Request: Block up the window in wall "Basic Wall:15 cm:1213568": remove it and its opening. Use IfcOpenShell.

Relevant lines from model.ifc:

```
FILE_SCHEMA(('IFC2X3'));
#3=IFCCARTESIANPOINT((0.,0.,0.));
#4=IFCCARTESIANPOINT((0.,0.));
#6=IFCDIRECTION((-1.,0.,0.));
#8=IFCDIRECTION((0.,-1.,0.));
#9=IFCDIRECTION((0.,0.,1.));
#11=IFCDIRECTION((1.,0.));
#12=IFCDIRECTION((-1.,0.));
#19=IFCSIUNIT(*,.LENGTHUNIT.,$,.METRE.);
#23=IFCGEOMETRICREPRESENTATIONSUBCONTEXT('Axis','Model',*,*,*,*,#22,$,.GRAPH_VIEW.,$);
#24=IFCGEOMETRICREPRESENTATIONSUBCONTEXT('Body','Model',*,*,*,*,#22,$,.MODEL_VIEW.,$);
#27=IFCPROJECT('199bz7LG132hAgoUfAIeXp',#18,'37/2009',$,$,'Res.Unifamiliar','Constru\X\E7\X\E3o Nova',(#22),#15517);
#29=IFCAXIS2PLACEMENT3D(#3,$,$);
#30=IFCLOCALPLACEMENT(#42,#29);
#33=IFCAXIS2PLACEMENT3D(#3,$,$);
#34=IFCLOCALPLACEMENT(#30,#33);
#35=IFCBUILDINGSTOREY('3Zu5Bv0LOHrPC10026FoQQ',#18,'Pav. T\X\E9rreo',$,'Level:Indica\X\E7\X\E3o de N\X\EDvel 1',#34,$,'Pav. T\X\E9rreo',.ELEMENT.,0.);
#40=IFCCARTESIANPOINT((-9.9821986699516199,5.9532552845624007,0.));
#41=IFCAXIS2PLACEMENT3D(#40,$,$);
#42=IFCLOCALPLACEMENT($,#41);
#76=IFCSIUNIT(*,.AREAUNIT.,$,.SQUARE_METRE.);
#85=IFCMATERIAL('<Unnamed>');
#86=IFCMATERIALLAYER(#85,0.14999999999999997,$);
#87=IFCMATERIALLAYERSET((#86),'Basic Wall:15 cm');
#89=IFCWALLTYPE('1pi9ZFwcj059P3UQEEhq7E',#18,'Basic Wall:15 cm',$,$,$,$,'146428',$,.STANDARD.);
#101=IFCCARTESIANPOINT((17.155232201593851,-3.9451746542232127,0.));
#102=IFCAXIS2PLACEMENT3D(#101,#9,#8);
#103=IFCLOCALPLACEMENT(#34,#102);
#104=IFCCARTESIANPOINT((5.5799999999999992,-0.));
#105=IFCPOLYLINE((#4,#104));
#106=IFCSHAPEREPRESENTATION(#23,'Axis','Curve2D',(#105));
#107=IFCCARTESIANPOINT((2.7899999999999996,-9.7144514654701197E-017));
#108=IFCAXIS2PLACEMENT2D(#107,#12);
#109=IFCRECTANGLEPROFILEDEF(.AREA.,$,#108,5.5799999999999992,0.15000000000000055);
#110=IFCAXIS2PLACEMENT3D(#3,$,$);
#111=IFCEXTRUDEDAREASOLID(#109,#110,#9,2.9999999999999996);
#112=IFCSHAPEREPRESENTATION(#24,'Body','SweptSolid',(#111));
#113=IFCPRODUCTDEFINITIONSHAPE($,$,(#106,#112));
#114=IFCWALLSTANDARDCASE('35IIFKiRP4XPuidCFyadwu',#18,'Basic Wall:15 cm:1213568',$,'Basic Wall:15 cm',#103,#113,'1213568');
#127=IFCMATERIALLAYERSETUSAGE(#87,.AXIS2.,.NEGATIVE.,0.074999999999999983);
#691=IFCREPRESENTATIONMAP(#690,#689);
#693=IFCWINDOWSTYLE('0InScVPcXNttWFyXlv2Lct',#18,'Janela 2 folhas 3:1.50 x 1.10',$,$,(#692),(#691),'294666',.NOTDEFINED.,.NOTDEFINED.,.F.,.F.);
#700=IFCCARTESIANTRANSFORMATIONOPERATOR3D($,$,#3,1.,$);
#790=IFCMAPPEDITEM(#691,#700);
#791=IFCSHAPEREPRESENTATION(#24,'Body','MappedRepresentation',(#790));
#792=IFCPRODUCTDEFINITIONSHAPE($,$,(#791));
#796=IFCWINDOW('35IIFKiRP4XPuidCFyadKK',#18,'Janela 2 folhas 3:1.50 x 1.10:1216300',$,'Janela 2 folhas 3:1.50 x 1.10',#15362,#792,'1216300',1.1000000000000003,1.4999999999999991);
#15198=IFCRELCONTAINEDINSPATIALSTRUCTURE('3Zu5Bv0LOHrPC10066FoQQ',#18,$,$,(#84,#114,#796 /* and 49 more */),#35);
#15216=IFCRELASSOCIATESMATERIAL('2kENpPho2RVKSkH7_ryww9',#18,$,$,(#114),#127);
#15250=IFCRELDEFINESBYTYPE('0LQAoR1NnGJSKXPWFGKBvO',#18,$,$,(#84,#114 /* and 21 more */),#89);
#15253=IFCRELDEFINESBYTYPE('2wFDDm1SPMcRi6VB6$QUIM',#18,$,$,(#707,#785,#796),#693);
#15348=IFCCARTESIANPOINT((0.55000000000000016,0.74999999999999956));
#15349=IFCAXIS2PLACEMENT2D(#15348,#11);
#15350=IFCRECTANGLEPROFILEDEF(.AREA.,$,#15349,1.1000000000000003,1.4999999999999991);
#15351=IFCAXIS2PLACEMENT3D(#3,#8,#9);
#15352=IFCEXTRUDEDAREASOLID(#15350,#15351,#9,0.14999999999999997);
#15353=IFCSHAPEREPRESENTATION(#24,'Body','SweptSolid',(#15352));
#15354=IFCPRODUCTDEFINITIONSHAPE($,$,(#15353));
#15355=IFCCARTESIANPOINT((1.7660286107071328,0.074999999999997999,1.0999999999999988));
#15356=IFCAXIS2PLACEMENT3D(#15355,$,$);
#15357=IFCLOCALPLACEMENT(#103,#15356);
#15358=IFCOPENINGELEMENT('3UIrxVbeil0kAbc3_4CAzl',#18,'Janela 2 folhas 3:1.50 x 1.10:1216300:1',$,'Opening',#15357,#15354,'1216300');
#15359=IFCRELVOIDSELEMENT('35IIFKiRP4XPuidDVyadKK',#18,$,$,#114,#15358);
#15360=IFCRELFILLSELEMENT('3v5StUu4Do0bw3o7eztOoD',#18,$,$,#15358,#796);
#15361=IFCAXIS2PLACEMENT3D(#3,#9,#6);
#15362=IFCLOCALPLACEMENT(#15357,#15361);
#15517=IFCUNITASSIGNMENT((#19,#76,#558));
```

```python
import ifcopenshell
import ifcopenshell.api.feature
import ifcopenshell.api.root
import ifcopenshell.geom
import ifcopenshell.util.shape

model = ifcopenshell.open("model.ifc")
settings = ifcopenshell.geom.settings()


def volume(element):
    """Net volume in cubic metres, openings subtracted."""
    shape = ifcopenshell.geom.create_shape(settings, element)
    return ifcopenshell.util.shape.get_volume(shape.geometry)


window = model.by_id(796)
opening = window.FillsVoids[0].RelatingOpeningElement
wall = opening.VoidsElements[0].RelatingBuildingElement
before = volume(wall)

ifcopenshell.api.root.remove_product(model, product=window)
ifcopenshell.api.feature.remove_feature(model, feature=opening)

after = volume(wall)

print(f"wall volume {before:.3f} -> {after:.3f} m3")

model.write("model-out.ifc")
```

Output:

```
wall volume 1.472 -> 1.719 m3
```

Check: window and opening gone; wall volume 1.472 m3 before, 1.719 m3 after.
